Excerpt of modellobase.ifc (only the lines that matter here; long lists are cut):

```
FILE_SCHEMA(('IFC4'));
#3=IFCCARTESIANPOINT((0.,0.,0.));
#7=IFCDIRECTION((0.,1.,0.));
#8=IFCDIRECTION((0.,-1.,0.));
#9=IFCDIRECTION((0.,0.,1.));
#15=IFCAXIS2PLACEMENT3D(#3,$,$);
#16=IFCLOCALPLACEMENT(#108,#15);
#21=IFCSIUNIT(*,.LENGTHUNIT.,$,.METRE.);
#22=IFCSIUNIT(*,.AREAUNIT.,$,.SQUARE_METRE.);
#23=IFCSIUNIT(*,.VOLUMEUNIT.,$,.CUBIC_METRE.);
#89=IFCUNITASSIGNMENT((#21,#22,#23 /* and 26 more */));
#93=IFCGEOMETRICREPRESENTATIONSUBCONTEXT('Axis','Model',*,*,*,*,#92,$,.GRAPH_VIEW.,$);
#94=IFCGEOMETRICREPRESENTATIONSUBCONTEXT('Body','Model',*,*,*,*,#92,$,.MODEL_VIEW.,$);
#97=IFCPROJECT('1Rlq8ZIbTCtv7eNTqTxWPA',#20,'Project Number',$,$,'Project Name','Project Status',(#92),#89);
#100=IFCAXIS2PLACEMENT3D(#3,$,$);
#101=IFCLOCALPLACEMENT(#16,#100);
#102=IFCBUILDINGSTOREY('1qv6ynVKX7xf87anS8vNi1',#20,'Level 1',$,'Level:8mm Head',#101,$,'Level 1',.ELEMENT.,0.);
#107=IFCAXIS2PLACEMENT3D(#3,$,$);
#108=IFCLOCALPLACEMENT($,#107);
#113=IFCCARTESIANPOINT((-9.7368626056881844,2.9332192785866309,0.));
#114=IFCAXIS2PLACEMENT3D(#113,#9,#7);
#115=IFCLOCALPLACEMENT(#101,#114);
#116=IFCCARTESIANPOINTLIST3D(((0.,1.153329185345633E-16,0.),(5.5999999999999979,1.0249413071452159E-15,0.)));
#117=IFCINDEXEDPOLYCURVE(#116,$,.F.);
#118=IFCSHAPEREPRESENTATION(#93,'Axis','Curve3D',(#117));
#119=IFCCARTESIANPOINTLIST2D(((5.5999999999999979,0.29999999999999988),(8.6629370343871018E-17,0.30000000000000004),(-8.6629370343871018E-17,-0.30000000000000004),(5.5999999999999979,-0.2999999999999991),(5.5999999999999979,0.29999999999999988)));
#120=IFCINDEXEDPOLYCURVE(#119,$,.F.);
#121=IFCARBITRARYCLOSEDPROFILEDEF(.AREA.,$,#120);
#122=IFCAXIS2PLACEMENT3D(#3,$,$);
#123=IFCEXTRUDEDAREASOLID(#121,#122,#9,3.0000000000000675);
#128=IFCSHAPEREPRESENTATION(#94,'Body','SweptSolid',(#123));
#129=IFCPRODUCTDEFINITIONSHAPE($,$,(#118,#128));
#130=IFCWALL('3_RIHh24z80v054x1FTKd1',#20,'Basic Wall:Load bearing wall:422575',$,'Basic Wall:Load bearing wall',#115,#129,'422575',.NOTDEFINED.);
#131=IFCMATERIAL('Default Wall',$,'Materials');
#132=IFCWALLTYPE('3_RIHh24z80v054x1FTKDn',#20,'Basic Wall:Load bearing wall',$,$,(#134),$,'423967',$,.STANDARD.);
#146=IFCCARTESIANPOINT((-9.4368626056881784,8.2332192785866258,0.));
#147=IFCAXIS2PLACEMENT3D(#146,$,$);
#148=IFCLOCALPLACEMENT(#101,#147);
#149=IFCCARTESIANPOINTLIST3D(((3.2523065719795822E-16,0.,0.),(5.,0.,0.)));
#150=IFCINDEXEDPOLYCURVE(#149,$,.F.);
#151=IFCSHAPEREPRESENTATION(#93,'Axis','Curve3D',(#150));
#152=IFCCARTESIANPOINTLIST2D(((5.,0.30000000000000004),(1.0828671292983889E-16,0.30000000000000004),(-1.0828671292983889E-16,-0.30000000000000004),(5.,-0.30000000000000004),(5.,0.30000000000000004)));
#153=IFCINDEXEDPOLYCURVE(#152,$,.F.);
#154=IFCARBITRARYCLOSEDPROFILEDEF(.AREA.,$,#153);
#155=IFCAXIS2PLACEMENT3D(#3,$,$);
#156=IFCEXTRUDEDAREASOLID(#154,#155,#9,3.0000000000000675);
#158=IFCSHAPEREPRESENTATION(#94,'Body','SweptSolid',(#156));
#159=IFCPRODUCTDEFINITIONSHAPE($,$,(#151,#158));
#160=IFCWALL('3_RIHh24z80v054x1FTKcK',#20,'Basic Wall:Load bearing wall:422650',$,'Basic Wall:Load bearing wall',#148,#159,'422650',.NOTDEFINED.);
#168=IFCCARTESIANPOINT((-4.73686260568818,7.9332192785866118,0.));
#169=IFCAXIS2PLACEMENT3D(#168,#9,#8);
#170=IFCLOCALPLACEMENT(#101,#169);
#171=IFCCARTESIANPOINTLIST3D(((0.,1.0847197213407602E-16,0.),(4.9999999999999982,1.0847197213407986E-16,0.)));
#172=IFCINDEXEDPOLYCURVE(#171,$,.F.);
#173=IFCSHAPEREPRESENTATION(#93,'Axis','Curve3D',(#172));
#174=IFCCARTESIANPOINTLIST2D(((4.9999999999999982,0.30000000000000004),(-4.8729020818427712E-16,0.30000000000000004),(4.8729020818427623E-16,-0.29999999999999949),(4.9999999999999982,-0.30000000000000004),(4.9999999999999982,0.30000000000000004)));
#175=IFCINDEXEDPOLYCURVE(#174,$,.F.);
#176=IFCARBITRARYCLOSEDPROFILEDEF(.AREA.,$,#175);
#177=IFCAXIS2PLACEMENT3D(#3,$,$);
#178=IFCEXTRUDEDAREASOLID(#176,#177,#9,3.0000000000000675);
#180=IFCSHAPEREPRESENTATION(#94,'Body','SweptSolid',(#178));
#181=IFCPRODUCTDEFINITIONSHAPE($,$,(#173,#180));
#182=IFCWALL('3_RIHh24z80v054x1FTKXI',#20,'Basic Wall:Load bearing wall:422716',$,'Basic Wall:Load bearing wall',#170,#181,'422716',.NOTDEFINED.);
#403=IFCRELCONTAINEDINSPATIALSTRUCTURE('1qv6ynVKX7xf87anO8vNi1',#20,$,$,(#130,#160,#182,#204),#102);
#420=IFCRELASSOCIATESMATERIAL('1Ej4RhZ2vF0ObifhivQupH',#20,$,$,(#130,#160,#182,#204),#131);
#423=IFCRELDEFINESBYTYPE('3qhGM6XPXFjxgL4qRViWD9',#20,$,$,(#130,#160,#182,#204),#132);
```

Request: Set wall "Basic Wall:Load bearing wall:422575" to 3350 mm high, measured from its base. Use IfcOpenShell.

```python
import ifcopenshell
import ifcopenshell.geom
import ifcopenshell.util.representation
import ifcopenshell.util.shape

model = ifcopenshell.open("modellobase.ifc")
settings = ifcopenshell.geom.settings()


def volume(element):
    """Net volume in cubic metres, openings subtracted."""
    shape = ifcopenshell.geom.create_shape(settings, element)
    return ifcopenshell.util.shape.get_volume(shape.geometry)


wall = model.by_guid("3_RIHh24z80v054x1FTKd1")
before = volume(wall)

body = ifcopenshell.util.representation.get_representation(wall, "Model", "Body")
solid = body.Items[0]
old_height = solid.Depth
solid.Depth = 3.35
after = volume(wall)

print(f"height {old_height:g} -> {solid.Depth:g}, volume {before:.3f} -> {after:.3f} m3")

model.write("modellobase_edited.ifc")
```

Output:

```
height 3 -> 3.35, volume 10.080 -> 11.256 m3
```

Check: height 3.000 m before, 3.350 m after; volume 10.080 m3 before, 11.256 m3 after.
